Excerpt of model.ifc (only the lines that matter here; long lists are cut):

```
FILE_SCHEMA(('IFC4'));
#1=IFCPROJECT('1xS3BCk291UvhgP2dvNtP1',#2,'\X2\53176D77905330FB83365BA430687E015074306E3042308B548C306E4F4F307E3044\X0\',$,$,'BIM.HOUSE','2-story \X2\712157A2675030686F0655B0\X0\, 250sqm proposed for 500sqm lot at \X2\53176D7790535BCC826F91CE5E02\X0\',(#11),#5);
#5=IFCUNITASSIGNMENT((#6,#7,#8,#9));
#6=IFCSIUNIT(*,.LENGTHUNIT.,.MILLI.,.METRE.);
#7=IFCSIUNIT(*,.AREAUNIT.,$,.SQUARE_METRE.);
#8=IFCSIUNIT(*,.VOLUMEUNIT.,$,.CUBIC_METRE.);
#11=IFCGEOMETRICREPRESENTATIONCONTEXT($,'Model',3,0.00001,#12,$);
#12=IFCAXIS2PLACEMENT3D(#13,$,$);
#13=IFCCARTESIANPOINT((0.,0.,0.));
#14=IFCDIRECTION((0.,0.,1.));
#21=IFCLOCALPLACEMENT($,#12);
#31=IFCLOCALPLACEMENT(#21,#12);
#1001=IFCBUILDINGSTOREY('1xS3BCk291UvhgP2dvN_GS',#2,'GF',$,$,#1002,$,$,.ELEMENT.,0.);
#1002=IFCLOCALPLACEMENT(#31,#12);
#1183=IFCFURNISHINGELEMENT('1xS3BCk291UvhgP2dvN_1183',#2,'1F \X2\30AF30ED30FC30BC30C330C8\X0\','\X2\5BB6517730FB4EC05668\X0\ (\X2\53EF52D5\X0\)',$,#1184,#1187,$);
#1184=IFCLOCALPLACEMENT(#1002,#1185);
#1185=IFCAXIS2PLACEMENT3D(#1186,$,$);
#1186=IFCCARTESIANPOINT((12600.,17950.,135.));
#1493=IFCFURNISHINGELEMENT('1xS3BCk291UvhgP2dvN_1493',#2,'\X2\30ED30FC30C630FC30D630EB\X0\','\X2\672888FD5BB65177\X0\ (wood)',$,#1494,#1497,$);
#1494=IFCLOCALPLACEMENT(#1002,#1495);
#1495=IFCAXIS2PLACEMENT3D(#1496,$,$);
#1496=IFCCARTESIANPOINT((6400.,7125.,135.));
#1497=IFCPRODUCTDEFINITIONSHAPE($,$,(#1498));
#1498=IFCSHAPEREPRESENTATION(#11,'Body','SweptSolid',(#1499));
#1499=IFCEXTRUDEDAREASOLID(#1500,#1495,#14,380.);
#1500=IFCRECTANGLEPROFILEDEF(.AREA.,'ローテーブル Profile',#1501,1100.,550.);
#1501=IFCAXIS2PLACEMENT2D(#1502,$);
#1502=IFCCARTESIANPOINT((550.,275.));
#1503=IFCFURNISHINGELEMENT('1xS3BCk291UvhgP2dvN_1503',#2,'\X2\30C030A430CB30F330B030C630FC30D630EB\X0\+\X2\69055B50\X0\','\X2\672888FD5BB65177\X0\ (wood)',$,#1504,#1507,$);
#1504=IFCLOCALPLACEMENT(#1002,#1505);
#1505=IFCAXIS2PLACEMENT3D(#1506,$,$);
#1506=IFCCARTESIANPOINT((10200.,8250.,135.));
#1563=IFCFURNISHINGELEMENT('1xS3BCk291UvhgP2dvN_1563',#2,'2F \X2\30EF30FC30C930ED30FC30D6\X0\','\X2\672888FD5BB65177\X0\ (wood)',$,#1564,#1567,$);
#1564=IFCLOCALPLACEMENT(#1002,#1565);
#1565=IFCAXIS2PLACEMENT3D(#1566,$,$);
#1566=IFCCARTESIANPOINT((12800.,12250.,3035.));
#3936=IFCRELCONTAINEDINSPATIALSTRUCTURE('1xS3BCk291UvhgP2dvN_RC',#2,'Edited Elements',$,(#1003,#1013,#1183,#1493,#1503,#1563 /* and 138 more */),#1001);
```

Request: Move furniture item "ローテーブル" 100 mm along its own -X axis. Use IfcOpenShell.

```python
import ifcopenshell
import ifcopenshell.api.geometry
import ifcopenshell.util.placement
import ifcopenshell.util.unit

model = ifcopenshell.open("model.ifc")
unit_scale = ifcopenshell.util.unit.calculate_unit_scale(model)

item = model.by_guid("1xS3BCk291UvhgP2dvN_1493")
matrix = ifcopenshell.util.placement.get_local_placement(item.ObjectPlacement)
matrix[:3, 3] -= matrix[:3, 0] * 0.1 / unit_scale
ifcopenshell.api.geometry.edit_object_placement(model, product=item, matrix=matrix, is_si=False)

print(ifcopenshell.util.placement.get_local_placement(item.ObjectPlacement).round(3) + 0.0)

model.write("model-out.ifc")
```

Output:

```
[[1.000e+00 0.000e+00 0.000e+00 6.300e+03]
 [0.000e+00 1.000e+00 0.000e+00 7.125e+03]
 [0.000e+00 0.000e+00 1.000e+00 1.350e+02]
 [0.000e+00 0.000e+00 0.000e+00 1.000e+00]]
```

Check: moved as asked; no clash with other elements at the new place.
